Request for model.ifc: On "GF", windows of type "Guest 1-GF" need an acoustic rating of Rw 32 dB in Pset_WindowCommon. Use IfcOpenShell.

First a look at what the model holds.

```python
import ifcopenshell
import ifcopenshell.util.element

model = ifcopenshell.open("model.ifc")
print(model.schema)
storey = next(s for s in model.by_type("IfcBuildingStorey") if s.Name == "GF")
windows = [e for e in ifcopenshell.util.element.get_decomposition(storey) if e.is_a("IfcWindow")]
seen = {}
for e in windows:
    element_type = ifcopenshell.util.element.get_type(e)
    key = (element_type.Name if element_type != e and element_type else None, ifcopenshell.util.element.get_pset(e, "Pset_WindowCommon", "AcousticRating"))
    seen[key] = seen.get(key, 0) + 1
for (name, value), count in sorted(seen.items(), key=str):
    print(count, "x", name, "|", value)
```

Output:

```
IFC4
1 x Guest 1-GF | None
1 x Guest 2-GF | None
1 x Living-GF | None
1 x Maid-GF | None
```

```python
import ifcopenshell
import ifcopenshell.api.pset
import ifcopenshell.util.element

model = ifcopenshell.open("model.ifc")

storey = next(s for s in model.by_type("IfcBuildingStorey") if s.Name == "GF")
windows = [e for e in ifcopenshell.util.element.get_decomposition(storey) if e.is_a("IfcWindow")]

count = 0
for e in windows:
    element_type = ifcopenshell.util.element.get_type(e)
    if element_type in (None, e) or element_type.Name != "Guest 1-GF":
        continue
    # add_pset returns the element's existing set when there is one.
    pset = ifcopenshell.api.pset.add_pset(model, product=e, name="Pset_WindowCommon")
    ifcopenshell.api.pset.edit_pset(model, pset=pset, properties={"AcousticRating": "Rw 32 dB"})
    count += 1

print(count, "windows updated")

model.write("model_v2.ifc")
```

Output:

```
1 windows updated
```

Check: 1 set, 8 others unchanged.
